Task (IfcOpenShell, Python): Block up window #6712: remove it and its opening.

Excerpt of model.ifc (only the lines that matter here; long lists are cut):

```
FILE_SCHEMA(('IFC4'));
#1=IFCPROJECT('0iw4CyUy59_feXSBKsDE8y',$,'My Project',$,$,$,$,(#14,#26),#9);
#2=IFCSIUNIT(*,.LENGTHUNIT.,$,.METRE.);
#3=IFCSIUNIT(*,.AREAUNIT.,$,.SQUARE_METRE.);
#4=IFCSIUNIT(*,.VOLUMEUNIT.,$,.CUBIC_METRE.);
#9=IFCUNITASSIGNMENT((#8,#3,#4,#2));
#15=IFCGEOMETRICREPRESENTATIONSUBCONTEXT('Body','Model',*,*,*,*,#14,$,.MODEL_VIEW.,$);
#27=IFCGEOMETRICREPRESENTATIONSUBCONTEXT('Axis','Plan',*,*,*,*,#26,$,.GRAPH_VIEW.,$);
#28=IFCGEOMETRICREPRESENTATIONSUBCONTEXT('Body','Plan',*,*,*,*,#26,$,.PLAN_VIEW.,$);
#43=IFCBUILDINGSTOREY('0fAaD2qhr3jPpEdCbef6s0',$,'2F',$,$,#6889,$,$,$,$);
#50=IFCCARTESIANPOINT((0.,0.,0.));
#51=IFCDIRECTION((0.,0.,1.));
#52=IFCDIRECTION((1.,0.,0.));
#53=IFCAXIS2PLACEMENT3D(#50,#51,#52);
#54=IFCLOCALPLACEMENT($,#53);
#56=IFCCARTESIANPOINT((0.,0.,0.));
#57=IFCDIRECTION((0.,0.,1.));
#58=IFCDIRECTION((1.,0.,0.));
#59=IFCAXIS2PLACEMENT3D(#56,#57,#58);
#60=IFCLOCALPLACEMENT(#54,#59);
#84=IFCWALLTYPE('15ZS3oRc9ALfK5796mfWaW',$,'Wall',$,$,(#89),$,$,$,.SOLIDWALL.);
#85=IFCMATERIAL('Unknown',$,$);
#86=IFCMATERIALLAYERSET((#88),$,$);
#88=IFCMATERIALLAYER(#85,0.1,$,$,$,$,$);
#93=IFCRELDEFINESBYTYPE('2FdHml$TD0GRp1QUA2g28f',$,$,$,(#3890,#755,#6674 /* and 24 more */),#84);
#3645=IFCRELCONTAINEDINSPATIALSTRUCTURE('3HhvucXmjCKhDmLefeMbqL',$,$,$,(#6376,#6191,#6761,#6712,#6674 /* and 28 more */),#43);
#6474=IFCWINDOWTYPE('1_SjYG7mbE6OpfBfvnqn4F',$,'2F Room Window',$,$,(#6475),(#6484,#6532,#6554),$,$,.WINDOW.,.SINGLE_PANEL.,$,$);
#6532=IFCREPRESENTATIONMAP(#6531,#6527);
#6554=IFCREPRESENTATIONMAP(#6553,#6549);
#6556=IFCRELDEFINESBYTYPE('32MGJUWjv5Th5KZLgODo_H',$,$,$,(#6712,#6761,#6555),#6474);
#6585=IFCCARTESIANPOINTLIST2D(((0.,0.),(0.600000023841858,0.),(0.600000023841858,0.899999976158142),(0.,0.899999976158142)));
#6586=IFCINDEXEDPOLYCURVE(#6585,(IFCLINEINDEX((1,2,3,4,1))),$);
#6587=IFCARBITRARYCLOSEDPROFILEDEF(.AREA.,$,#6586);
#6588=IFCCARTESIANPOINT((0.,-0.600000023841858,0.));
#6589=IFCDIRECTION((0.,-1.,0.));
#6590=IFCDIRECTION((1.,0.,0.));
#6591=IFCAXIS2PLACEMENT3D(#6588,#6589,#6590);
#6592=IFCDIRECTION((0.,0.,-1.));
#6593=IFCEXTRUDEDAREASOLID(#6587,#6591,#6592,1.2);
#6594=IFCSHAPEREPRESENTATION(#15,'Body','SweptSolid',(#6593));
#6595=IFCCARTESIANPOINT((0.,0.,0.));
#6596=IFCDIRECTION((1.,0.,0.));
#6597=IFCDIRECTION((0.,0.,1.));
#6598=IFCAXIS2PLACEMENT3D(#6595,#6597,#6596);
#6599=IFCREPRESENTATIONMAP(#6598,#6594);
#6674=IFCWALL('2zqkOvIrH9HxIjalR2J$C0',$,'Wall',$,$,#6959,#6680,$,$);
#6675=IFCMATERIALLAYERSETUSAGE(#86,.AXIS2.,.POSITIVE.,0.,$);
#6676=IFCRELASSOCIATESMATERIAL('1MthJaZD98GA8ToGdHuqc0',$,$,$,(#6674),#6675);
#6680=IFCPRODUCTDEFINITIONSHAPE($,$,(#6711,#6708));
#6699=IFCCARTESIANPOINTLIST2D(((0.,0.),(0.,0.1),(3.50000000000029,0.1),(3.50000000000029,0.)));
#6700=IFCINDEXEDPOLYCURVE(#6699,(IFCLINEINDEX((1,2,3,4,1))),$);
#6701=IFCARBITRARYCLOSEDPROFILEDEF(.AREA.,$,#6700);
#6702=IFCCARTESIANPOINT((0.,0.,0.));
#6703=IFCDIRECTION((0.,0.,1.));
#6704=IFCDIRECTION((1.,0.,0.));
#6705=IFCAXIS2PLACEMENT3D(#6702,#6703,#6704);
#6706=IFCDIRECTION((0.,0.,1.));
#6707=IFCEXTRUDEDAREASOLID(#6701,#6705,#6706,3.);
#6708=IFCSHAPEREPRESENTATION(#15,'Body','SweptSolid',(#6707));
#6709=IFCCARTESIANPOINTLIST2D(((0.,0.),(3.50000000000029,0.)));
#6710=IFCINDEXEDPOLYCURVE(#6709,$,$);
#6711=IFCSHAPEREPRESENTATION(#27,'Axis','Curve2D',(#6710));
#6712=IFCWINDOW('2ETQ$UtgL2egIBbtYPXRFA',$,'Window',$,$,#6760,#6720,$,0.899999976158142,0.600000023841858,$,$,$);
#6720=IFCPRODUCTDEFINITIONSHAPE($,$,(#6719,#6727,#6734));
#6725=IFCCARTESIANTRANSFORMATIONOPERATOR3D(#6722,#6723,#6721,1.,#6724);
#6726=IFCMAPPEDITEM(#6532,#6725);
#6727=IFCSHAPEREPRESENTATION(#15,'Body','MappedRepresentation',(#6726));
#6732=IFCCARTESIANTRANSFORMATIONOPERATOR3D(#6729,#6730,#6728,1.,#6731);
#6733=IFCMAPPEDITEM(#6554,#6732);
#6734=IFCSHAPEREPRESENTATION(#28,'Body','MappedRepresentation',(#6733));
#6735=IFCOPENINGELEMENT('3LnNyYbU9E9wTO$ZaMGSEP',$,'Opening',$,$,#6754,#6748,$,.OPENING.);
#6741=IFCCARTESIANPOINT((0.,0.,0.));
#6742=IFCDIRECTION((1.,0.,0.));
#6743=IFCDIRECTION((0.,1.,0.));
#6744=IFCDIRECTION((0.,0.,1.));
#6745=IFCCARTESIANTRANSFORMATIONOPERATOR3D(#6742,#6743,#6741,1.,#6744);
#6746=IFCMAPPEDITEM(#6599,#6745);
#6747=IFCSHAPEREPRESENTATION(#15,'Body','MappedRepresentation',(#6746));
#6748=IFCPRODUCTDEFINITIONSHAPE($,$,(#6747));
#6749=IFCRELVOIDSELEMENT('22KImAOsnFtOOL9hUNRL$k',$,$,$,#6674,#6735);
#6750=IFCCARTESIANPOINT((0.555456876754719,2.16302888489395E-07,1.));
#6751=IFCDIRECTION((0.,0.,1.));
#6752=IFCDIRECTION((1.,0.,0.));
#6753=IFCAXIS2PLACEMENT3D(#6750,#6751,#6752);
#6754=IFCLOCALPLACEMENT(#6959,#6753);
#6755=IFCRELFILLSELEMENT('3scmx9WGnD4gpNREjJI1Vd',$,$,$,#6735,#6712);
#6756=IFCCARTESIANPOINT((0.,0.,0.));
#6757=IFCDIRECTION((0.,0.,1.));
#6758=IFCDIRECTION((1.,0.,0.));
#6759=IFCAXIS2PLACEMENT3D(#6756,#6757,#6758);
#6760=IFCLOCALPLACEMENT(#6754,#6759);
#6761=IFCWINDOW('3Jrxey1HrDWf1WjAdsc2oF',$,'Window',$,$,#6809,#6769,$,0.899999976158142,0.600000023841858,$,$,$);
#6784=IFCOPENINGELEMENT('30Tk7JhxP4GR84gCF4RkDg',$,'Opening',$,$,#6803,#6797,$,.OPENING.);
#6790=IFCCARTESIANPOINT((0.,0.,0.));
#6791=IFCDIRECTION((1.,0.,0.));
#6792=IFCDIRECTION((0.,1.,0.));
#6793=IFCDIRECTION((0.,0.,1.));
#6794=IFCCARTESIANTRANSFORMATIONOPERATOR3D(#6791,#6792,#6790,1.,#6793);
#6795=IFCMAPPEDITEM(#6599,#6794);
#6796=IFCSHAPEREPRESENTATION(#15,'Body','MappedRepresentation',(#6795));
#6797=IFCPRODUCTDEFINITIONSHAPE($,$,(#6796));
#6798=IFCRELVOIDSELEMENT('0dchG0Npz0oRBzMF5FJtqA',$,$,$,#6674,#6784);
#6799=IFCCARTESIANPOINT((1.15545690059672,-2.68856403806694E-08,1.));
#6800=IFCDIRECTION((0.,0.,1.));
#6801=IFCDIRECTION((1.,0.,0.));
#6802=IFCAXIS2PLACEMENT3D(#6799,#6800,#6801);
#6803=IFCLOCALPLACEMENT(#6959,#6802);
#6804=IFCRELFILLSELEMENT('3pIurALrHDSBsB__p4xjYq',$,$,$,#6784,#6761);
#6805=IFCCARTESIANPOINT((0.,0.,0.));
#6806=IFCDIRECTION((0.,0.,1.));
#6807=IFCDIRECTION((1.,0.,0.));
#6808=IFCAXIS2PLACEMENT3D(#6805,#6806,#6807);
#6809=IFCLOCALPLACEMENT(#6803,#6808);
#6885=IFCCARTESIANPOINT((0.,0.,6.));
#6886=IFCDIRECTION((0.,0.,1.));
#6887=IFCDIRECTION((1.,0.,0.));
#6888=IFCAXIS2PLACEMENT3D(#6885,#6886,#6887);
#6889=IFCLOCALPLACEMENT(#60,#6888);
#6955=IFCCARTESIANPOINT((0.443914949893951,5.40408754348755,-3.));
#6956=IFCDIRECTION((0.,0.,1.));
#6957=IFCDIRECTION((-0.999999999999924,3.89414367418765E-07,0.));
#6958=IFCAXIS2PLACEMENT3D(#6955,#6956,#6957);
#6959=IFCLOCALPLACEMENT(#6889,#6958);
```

```python
import ifcopenshell
import ifcopenshell.api.feature
import ifcopenshell.api.root
import ifcopenshell.geom
import ifcopenshell.util.shape

model = ifcopenshell.open("model.ifc")
settings = ifcopenshell.geom.settings()


def volume(element):
    """Net volume in cubic metres, openings subtracted."""
    shape = ifcopenshell.geom.create_shape(settings, element)
    return ifcopenshell.util.shape.get_volume(shape.geometry)


window = model.by_id(6712)
opening = window.FillsVoids[0].RelatingOpeningElement
wall = opening.VoidsElements[0].RelatingBuildingElement
before = volume(wall)

ifcopenshell.api.root.remove_product(model, product=window)
ifcopenshell.api.feature.remove_feature(model, feature=opening)

after = volume(wall)

print(f"wall volume {before:.3f} -> {after:.3f} m3")

model.write("model-out.ifc")
```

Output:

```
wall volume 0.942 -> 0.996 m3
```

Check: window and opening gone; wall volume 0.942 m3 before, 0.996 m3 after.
